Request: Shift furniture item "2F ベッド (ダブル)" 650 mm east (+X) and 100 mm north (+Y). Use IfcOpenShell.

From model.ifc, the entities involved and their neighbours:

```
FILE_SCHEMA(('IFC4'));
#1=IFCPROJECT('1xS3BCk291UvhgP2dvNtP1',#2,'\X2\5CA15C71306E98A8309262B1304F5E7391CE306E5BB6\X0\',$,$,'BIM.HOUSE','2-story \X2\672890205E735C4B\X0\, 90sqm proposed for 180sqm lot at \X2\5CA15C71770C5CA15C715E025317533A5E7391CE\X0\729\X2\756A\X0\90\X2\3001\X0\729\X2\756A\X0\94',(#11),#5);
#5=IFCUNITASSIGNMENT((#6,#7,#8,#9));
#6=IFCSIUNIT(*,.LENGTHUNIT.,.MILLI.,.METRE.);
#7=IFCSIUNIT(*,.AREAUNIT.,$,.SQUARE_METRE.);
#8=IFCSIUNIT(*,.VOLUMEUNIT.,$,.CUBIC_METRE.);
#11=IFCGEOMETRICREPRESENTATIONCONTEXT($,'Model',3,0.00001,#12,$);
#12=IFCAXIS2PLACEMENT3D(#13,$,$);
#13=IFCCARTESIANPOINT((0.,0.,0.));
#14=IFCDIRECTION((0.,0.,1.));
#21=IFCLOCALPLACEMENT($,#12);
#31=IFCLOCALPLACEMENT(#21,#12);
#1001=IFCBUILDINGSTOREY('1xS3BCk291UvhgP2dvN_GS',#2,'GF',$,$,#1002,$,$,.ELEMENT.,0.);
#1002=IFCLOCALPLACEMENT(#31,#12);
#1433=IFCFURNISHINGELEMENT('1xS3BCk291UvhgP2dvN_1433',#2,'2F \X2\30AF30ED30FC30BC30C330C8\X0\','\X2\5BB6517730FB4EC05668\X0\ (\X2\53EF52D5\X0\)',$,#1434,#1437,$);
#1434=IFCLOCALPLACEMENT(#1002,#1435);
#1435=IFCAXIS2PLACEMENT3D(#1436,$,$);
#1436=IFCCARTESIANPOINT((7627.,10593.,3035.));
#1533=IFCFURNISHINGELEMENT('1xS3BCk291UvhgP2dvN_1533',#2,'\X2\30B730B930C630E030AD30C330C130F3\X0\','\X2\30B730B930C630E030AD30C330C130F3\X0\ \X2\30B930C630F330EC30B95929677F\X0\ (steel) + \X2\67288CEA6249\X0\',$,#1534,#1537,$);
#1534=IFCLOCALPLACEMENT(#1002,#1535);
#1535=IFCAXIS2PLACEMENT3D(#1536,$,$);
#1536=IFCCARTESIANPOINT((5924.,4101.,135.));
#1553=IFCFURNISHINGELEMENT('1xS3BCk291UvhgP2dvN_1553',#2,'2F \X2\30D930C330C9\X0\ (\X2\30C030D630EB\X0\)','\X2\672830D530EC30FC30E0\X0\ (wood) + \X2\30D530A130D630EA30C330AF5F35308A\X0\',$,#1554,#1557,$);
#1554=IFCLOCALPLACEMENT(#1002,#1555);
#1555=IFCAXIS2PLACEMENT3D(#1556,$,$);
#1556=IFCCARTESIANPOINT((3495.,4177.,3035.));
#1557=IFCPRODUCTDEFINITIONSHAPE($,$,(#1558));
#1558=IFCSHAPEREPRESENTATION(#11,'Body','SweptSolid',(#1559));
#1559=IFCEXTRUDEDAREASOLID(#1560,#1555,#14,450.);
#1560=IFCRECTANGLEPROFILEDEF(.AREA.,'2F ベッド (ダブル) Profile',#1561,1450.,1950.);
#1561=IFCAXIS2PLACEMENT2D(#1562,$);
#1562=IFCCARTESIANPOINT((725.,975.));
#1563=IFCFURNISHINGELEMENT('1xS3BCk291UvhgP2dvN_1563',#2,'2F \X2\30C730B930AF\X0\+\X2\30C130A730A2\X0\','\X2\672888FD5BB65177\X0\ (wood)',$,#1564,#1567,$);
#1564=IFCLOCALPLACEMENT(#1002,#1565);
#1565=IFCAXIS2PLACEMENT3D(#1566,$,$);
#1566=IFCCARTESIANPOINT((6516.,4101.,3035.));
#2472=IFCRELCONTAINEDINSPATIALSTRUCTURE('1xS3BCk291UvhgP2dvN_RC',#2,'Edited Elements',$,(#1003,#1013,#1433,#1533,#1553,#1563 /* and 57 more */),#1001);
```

```python
import ifcopenshell
import ifcopenshell.api.geometry
import ifcopenshell.util.placement
import ifcopenshell.util.unit

model = ifcopenshell.open("model.ifc")
unit_scale = ifcopenshell.util.unit.calculate_unit_scale(model)

item = model.by_guid("1xS3BCk291UvhgP2dvN_1553")
matrix = ifcopenshell.util.placement.get_local_placement(item.ObjectPlacement)
matrix[0, 3] += 0.65 / unit_scale
matrix[1, 3] += 0.1 / unit_scale
ifcopenshell.api.geometry.edit_object_placement(model, product=item, matrix=matrix, is_si=False)

print(ifcopenshell.util.placement.get_local_placement(item.ObjectPlacement).round(3) + 0.0)

model.write("model-out.ifc")
```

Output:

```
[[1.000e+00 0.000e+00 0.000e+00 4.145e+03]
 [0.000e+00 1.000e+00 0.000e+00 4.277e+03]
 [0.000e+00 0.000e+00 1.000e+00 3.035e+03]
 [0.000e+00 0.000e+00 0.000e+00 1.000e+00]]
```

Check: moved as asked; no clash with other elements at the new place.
